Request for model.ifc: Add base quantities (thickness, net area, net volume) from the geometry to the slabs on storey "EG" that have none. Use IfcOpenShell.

First a look at what the model holds.

```python
import ifcopenshell
import ifcopenshell.util.element
import ifcopenshell.util.unit

model = ifcopenshell.open("model.ifc")
print(model.schema)
for unit_type in ("LENGTHUNIT", "AREAUNIT", "VOLUMEUNIT"):
    print(unit_type, ifcopenshell.util.unit.calculate_unit_scale(model, unit_type))
storey = next(s for s in model.by_type("IfcBuildingStorey") if s.Name == "EG")
slabs = [e for e in ifcopenshell.util.element.get_decomposition(storey) if e.is_a("IfcSlab")]
for e in sorted(slabs, key=lambda e: e.id()):
    print(e.id(), e.is_a(), e.Name, list(ifcopenshell.util.element.get_psets(e, qtos_only=True)), sep=" | ")
```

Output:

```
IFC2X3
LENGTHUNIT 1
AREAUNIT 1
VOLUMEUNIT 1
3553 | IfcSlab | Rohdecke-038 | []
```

```python
import ifcopenshell
import ifcopenshell.api.pset
import ifcopenshell.geom
import ifcopenshell.util.element
import ifcopenshell.util.shape
import ifcopenshell.util.unit

model = ifcopenshell.open("model.ifc")
unit_scale = ifcopenshell.util.unit.calculate_unit_scale(model)
area_scale = ifcopenshell.util.unit.calculate_unit_scale(model, "AREAUNIT")
volume_scale = ifcopenshell.util.unit.calculate_unit_scale(model, "VOLUMEUNIT")
settings = ifcopenshell.geom.settings()

storey = next(s for s in model.by_type("IfcBuildingStorey") if s.Name == "EG")
slabs = [e for e in ifcopenshell.util.element.get_decomposition(storey) if e.is_a("IfcSlab")]

for e in sorted(slabs, key=lambda e: e.id()):
    if ifcopenshell.util.element.get_psets(e, qtos_only=True, should_inherit=False):
        continue
    # Geometry comes back in metres, in the element's own axes.
    shape = ifcopenshell.geom.create_shape(settings, e)
    values = {
        "Width": ifcopenshell.util.shape.get_z(shape.geometry) / unit_scale,
        "NetArea": ifcopenshell.util.shape.get_footprint_area(shape.geometry) / area_scale,
        "NetVolume": ifcopenshell.util.shape.get_volume(shape.geometry) / volume_scale,
    }
    qto = ifcopenshell.api.pset.add_qto(model, product=e, name="BaseQuantities")
    ifcopenshell.api.pset.edit_qto(model, qto=qto, properties=values)
    print(e.id(), {k: round(v, 3) for k, v in values.items()})

model.write("model_v2.ifc")
```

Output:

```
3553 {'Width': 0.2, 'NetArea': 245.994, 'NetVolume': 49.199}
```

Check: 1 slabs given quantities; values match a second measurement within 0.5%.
